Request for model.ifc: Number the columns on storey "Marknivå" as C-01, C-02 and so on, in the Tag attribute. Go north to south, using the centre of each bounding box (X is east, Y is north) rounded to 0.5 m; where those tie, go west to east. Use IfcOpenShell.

First a look at what the model holds.

```python
import ifcopenshell
import ifcopenshell.util.element
import ifcopenshell.util.placement

model = ifcopenshell.open("model.ifc")
print(model.schema)
storey = next(s for s in model.by_type("IfcBuildingStorey") if s.Name == "Marknivå")
columns = [e for e in ifcopenshell.util.element.get_decomposition(storey) if e.is_a("IfcColumn")]
for e in sorted(columns, key=lambda e: e.id()):
    origin = ifcopenshell.util.placement.get_local_placement(e.ObjectPlacement)[:3, 3]
    print(e.id(), e.Tag, e.Name, origin.round(2) + 0.0, sep=" | ")
```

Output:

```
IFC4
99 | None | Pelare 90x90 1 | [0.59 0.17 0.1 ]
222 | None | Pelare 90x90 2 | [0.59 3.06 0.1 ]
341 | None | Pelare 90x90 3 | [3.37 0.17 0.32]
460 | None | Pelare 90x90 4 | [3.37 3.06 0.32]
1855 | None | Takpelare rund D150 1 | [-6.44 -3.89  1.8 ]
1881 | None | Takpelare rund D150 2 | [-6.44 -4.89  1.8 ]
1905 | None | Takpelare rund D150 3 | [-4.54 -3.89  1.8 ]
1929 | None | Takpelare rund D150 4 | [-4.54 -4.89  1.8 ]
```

```python
import ifcopenshell
import ifcopenshell.geom
import ifcopenshell.util.element
import ifcopenshell.util.shape

model = ifcopenshell.open("model.ifc")
settings = ifcopenshell.geom.settings()
settings.set("use-world-coords", True)


def centre(element):
    shape = ifcopenshell.geom.create_shape(settings, element)
    return ifcopenshell.util.shape.get_bbox_centroid(shape.geometry)


storey = next(s for s in model.by_type("IfcBuildingStorey") if s.Name == "Marknivå")
columns = [e for e in ifcopenshell.util.element.get_decomposition(storey) if e.is_a("IfcColumn")]

# Insertion points can sit at a corner or the storey origin, so sort by the geometry (in metres).
centres = {e: centre(e) for e in columns}
columns.sort(key=lambda e: (-round(centres[e][1] / 0.5), centres[e][0]))

for i, e in enumerate(columns, start=1):
    number = f"C-{i:02d}"
    e.Tag = number
    print(e.id(), number)

model.write("model_rev.ifc")
```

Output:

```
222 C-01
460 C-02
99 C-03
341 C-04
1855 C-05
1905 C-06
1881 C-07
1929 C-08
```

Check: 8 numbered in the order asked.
